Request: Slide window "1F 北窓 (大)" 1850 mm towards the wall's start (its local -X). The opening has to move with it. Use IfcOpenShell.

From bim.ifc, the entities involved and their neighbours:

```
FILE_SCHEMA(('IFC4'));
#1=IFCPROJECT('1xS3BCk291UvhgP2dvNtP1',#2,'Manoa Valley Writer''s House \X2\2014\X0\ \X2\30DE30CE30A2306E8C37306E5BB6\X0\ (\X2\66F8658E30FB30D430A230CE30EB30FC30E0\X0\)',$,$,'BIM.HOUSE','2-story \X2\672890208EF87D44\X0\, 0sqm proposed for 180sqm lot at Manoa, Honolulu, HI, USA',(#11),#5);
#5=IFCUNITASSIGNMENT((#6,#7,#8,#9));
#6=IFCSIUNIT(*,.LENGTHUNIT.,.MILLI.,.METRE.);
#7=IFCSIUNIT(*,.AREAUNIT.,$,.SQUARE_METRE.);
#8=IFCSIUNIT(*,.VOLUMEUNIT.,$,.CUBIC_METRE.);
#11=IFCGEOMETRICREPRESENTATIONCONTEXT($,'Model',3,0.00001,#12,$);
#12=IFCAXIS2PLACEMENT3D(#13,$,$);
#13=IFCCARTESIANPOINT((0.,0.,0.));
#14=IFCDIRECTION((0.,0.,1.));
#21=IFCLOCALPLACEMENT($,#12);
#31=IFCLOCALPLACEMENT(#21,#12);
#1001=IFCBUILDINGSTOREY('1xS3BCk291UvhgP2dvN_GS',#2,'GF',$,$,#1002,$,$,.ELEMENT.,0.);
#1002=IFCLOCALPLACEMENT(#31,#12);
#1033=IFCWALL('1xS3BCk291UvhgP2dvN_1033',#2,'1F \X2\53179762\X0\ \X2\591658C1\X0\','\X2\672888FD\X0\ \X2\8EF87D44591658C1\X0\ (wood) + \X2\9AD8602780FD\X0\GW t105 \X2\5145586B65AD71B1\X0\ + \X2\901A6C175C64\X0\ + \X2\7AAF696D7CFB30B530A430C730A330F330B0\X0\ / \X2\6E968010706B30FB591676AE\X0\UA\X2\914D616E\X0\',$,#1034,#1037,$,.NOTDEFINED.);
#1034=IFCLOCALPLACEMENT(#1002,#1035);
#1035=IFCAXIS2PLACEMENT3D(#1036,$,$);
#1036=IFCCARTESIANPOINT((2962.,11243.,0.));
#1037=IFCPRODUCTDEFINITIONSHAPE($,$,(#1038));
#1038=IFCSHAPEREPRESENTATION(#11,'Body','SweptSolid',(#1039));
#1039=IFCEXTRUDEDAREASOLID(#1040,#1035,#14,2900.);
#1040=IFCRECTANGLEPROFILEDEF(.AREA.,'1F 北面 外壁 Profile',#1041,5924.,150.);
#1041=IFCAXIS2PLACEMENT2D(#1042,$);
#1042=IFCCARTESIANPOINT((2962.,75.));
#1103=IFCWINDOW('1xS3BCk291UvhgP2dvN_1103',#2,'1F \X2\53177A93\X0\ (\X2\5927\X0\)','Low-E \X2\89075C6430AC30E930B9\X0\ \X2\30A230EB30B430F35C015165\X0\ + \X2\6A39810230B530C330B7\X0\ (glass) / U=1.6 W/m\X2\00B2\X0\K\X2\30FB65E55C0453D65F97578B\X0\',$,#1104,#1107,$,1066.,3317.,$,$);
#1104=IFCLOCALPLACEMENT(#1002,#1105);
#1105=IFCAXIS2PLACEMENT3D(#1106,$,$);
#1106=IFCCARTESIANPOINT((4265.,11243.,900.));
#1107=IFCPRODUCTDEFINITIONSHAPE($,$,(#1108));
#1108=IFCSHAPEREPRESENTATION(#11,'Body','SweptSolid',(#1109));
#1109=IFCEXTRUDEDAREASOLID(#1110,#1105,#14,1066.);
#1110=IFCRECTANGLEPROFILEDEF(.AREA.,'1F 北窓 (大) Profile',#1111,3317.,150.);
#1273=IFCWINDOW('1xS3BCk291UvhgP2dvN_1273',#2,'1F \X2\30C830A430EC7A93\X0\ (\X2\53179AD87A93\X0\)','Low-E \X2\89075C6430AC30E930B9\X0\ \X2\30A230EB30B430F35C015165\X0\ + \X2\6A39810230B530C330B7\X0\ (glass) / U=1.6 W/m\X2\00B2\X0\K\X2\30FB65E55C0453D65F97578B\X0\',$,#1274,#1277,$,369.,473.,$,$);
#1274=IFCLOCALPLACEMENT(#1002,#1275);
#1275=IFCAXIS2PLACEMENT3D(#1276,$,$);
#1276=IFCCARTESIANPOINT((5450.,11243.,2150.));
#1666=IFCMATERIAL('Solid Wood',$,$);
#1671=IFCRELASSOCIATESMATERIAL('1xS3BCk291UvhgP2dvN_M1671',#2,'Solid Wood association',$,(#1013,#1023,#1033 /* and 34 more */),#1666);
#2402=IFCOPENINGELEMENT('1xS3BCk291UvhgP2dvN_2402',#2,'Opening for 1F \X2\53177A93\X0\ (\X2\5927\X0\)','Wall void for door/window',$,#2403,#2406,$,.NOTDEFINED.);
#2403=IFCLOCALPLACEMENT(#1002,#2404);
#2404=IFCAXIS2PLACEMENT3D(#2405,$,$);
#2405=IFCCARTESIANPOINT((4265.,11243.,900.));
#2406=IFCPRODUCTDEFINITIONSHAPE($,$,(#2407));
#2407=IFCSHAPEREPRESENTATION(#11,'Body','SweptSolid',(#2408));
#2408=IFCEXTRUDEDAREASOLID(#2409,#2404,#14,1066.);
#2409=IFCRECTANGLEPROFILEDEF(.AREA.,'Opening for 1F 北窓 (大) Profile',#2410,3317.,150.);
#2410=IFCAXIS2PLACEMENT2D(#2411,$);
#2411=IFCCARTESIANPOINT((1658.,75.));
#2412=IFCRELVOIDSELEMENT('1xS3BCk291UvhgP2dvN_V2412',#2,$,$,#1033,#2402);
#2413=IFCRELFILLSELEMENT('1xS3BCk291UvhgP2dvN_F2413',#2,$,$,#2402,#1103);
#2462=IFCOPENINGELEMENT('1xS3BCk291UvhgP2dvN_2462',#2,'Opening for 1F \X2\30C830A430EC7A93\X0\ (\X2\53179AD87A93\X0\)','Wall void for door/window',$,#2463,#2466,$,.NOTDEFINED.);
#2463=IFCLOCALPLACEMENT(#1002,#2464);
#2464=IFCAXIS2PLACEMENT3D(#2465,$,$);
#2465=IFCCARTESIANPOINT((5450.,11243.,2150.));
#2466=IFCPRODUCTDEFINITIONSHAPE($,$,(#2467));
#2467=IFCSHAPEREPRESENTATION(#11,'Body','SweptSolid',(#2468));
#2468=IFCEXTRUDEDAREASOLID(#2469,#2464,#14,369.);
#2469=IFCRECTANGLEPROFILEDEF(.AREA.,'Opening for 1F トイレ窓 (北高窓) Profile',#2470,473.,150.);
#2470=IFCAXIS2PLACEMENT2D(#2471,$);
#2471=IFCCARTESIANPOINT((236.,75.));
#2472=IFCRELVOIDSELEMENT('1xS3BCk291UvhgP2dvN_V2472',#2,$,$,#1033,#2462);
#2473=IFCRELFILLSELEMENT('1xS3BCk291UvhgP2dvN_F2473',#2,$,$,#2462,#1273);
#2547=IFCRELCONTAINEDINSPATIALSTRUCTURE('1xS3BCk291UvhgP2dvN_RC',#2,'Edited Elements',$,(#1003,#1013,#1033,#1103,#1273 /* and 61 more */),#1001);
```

```python
import ifcopenshell
import ifcopenshell.api.geometry
import ifcopenshell.util.placement

model = ifcopenshell.open("bim.ifc")

window = model.by_guid("1xS3BCk291UvhgP2dvN_1103")
opening = window.FillsVoids[0].RelatingOpeningElement
wall = opening.VoidsElements[0].RelatingBuildingElement

wall_matrix = ifcopenshell.util.placement.get_local_placement(wall.ObjectPlacement)
shift = wall_matrix[:3, 0] * -1850.0
before = ifcopenshell.util.placement.get_local_placement(window.ObjectPlacement)[:3, 3].copy()

# The window is not placed relative to its opening, so move both.
for product in (opening, window):
    matrix = ifcopenshell.util.placement.get_local_placement(product.ObjectPlacement)
    matrix[:3, 3] += shift
    ifcopenshell.api.geometry.edit_object_placement(model, product=product, matrix=matrix, is_si=False)

after = ifcopenshell.util.placement.get_local_placement(window.ObjectPlacement)[:3, 3]
print("window moved by", (after - before).round(3) + 0.0)

model.write("bim_updated.ifc")
```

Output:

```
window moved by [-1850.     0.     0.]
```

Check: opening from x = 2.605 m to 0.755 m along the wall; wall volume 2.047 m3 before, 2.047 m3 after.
